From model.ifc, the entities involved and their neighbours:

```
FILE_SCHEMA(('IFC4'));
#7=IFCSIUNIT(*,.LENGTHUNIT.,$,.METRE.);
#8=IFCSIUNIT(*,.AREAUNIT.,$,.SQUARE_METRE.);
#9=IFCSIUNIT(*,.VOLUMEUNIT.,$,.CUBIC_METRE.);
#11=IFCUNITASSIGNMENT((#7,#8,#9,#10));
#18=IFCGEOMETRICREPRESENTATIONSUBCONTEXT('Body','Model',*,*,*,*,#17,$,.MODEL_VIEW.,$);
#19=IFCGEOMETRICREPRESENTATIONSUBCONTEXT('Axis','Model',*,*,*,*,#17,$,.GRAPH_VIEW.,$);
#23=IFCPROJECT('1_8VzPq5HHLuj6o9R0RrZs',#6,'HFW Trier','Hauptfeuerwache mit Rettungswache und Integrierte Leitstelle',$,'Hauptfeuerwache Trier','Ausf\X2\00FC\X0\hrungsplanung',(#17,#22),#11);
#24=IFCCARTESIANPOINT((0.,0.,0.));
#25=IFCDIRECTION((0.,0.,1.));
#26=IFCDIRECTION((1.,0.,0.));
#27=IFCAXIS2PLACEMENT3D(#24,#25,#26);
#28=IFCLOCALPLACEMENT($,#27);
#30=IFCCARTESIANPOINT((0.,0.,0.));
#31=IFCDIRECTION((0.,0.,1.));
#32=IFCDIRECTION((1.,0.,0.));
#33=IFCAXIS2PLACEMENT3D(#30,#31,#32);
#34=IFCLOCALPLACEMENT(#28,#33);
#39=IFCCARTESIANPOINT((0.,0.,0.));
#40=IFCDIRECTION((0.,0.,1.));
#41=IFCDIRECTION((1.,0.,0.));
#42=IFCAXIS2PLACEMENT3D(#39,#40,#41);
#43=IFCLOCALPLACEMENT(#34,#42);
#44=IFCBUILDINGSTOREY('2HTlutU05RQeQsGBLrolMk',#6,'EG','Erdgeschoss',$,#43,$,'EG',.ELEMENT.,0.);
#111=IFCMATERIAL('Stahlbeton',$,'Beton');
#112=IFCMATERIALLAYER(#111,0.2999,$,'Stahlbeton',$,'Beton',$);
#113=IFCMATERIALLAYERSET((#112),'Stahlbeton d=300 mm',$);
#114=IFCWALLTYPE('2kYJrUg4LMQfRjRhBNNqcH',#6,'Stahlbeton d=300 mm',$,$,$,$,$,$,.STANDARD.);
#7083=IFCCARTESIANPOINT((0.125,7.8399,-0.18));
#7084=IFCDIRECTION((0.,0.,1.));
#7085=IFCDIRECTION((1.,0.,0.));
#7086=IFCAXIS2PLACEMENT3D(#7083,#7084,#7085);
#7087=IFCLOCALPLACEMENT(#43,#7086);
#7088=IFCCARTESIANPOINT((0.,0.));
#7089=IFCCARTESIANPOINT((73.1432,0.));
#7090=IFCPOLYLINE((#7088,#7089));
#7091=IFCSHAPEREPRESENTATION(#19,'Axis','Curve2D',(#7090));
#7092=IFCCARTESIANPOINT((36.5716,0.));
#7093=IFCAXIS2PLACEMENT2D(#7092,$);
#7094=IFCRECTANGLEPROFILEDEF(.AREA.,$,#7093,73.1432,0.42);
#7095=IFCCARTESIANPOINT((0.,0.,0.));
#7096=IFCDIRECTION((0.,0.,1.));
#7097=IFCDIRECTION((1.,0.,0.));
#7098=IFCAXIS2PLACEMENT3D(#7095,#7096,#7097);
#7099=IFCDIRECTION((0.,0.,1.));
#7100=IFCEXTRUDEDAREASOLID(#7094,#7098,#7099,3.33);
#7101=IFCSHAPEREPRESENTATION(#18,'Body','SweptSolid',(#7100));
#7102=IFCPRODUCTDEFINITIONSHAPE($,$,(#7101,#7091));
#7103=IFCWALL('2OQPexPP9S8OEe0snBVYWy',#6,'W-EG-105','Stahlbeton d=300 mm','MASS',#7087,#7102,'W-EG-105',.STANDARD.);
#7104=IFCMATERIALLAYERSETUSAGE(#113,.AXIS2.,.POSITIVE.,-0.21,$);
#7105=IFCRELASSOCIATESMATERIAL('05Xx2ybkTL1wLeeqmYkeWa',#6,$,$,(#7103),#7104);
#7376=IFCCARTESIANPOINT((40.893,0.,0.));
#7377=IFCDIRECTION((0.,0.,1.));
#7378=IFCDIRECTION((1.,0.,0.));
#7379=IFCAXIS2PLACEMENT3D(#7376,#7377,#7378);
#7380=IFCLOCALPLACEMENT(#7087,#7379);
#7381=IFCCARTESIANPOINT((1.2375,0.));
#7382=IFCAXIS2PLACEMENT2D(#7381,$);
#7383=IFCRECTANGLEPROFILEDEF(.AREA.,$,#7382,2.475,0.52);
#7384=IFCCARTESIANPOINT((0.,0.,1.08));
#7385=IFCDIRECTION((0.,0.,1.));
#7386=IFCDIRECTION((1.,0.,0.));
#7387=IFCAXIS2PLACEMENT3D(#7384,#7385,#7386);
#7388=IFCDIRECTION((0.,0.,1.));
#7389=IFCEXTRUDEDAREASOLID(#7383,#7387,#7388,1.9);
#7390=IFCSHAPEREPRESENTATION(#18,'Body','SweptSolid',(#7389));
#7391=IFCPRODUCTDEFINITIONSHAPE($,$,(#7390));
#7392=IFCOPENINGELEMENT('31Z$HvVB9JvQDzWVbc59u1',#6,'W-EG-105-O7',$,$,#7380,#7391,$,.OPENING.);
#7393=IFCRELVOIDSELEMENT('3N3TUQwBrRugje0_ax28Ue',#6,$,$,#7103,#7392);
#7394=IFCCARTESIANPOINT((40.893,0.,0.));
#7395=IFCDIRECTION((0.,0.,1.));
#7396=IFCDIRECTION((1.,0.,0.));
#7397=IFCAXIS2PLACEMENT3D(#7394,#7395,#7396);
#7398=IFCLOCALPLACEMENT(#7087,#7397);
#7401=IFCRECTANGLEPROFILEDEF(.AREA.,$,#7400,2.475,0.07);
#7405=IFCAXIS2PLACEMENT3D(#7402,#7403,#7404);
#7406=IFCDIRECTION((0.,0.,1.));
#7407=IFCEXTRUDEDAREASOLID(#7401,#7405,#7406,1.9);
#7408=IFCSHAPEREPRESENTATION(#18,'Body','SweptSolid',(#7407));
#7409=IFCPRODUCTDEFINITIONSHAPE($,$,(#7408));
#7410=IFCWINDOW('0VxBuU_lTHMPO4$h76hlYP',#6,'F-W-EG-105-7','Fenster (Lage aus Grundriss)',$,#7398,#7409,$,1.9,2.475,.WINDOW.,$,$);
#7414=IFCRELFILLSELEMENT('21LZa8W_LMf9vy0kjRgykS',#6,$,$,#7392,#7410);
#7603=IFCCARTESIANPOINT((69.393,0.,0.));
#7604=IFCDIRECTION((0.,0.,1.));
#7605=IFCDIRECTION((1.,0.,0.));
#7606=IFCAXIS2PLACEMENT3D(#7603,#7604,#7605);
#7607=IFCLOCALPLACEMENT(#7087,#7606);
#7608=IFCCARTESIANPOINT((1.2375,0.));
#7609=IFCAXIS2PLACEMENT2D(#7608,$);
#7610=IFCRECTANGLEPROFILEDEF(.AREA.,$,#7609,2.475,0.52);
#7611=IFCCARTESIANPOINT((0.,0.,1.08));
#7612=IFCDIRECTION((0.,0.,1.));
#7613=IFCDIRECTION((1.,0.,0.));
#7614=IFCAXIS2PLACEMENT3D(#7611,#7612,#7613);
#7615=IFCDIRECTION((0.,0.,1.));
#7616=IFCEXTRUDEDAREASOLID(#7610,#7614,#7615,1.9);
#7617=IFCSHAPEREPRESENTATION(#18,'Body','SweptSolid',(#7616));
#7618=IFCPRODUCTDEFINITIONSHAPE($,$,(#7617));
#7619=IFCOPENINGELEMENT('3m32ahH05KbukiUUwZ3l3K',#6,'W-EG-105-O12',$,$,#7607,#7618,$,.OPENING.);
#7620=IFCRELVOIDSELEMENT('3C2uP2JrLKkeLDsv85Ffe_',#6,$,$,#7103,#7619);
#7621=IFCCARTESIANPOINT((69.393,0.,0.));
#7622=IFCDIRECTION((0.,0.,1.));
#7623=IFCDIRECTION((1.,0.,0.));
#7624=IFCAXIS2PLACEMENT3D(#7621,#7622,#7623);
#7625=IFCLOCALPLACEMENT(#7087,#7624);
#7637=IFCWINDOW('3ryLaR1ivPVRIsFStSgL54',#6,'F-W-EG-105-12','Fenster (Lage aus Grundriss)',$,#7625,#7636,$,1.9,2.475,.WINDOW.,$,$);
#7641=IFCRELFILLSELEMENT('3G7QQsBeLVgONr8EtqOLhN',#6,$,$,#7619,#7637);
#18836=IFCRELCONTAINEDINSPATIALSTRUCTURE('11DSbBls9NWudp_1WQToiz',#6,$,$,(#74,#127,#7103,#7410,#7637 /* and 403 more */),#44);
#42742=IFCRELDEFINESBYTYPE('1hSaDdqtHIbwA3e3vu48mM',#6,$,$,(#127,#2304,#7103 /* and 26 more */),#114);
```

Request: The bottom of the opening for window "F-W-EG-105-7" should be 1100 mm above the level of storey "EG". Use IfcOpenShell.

```python
import numpy as np
import ifcopenshell
import ifcopenshell.api.geometry
import ifcopenshell.geom
import ifcopenshell.util.element
import ifcopenshell.util.placement
import ifcopenshell.util.shape
import ifcopenshell.util.unit

model = ifcopenshell.open("model.ifc")
unit_scale = ifcopenshell.util.unit.calculate_unit_scale(model)

window = model.by_guid("0VxBuU_lTHMPO4$h76hlYP")
opening = window.FillsVoids[0].RelatingOpeningElement
storey = ifcopenshell.util.element.get_container(window, ifc_class="IfcBuildingStorey")
level = ifcopenshell.util.placement.get_local_placement(storey.ObjectPlacement)[2, 3]

# The opening's origin need not be at the sill, so measure its lowest point.
shape = ifcopenshell.geom.create_shape(ifcopenshell.geom.settings(), opening)
bottom = ifcopenshell.util.shape.get_shape_bottom_elevation(shape, shape.geometry) / unit_scale
dz = level + 1.1 / unit_scale - bottom

shift = np.array([0.0, 0.0, dz])
# The window is not placed relative to its opening, so move both.
for product in (opening, window):
    matrix = ifcopenshell.util.placement.get_local_placement(product.ObjectPlacement)
    matrix[:3, 3] += shift
    ifcopenshell.api.geometry.edit_object_placement(model, product=product, matrix=matrix, is_si=False)

print(f"moved by {dz * unit_scale:+.3f} m")

model.write("model_updated.ifc")
```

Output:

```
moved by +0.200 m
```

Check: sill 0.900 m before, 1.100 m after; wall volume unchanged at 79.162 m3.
